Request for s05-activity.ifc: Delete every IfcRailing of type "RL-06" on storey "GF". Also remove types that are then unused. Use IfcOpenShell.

First a look at what the model holds.

```python
import ifcopenshell
import ifcopenshell.util.element

model = ifcopenshell.open("s05-activity.ifc")
print(model.schema)
storey = next(s for s in model.by_type("IfcBuildingStorey") if s.Name == "GF")
railings = [e for e in ifcopenshell.util.element.get_decomposition(storey) if e.is_a("IfcRailing")]
seen = {}
for e in railings:
    element_type = ifcopenshell.util.element.get_type(e)
    name = element_type.Name if element_type not in (None, e) else None
    seen[name] = seen.get(name, 0) + 1
for name, count in sorted(seen.items(), key=str):
    print(count, "x", name)
```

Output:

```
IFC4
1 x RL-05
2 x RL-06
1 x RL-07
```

```python
import ifcopenshell
import ifcopenshell.api.root
import ifcopenshell.util.element

model = ifcopenshell.open("s05-activity.ifc")

storey = next(s for s in model.by_type("IfcBuildingStorey") if s.Name == "GF")
railings = [e for e in ifcopenshell.util.element.get_decomposition(storey) if e.is_a("IfcRailing")]
targets = [e for e in railings if (t := ifcopenshell.util.element.get_type(e)) not in (None, e) and t.Name == "RL-06"]
types = {ifcopenshell.util.element.get_type(e) for e in targets} - {None, *targets}

for e in targets:
    ifcopenshell.api.root.remove_product(model, product=e)
print(len(targets), "removed")

unused = [t for t in types if not ifcopenshell.util.element.get_types(t)]
for t in unused:
    ifcopenshell.api.root.remove_product(model, product=t)
print(len(unused), "unused types removed")

model.write("s05-activity_edited.ifc")
```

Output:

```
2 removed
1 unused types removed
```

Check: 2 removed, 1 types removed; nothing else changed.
